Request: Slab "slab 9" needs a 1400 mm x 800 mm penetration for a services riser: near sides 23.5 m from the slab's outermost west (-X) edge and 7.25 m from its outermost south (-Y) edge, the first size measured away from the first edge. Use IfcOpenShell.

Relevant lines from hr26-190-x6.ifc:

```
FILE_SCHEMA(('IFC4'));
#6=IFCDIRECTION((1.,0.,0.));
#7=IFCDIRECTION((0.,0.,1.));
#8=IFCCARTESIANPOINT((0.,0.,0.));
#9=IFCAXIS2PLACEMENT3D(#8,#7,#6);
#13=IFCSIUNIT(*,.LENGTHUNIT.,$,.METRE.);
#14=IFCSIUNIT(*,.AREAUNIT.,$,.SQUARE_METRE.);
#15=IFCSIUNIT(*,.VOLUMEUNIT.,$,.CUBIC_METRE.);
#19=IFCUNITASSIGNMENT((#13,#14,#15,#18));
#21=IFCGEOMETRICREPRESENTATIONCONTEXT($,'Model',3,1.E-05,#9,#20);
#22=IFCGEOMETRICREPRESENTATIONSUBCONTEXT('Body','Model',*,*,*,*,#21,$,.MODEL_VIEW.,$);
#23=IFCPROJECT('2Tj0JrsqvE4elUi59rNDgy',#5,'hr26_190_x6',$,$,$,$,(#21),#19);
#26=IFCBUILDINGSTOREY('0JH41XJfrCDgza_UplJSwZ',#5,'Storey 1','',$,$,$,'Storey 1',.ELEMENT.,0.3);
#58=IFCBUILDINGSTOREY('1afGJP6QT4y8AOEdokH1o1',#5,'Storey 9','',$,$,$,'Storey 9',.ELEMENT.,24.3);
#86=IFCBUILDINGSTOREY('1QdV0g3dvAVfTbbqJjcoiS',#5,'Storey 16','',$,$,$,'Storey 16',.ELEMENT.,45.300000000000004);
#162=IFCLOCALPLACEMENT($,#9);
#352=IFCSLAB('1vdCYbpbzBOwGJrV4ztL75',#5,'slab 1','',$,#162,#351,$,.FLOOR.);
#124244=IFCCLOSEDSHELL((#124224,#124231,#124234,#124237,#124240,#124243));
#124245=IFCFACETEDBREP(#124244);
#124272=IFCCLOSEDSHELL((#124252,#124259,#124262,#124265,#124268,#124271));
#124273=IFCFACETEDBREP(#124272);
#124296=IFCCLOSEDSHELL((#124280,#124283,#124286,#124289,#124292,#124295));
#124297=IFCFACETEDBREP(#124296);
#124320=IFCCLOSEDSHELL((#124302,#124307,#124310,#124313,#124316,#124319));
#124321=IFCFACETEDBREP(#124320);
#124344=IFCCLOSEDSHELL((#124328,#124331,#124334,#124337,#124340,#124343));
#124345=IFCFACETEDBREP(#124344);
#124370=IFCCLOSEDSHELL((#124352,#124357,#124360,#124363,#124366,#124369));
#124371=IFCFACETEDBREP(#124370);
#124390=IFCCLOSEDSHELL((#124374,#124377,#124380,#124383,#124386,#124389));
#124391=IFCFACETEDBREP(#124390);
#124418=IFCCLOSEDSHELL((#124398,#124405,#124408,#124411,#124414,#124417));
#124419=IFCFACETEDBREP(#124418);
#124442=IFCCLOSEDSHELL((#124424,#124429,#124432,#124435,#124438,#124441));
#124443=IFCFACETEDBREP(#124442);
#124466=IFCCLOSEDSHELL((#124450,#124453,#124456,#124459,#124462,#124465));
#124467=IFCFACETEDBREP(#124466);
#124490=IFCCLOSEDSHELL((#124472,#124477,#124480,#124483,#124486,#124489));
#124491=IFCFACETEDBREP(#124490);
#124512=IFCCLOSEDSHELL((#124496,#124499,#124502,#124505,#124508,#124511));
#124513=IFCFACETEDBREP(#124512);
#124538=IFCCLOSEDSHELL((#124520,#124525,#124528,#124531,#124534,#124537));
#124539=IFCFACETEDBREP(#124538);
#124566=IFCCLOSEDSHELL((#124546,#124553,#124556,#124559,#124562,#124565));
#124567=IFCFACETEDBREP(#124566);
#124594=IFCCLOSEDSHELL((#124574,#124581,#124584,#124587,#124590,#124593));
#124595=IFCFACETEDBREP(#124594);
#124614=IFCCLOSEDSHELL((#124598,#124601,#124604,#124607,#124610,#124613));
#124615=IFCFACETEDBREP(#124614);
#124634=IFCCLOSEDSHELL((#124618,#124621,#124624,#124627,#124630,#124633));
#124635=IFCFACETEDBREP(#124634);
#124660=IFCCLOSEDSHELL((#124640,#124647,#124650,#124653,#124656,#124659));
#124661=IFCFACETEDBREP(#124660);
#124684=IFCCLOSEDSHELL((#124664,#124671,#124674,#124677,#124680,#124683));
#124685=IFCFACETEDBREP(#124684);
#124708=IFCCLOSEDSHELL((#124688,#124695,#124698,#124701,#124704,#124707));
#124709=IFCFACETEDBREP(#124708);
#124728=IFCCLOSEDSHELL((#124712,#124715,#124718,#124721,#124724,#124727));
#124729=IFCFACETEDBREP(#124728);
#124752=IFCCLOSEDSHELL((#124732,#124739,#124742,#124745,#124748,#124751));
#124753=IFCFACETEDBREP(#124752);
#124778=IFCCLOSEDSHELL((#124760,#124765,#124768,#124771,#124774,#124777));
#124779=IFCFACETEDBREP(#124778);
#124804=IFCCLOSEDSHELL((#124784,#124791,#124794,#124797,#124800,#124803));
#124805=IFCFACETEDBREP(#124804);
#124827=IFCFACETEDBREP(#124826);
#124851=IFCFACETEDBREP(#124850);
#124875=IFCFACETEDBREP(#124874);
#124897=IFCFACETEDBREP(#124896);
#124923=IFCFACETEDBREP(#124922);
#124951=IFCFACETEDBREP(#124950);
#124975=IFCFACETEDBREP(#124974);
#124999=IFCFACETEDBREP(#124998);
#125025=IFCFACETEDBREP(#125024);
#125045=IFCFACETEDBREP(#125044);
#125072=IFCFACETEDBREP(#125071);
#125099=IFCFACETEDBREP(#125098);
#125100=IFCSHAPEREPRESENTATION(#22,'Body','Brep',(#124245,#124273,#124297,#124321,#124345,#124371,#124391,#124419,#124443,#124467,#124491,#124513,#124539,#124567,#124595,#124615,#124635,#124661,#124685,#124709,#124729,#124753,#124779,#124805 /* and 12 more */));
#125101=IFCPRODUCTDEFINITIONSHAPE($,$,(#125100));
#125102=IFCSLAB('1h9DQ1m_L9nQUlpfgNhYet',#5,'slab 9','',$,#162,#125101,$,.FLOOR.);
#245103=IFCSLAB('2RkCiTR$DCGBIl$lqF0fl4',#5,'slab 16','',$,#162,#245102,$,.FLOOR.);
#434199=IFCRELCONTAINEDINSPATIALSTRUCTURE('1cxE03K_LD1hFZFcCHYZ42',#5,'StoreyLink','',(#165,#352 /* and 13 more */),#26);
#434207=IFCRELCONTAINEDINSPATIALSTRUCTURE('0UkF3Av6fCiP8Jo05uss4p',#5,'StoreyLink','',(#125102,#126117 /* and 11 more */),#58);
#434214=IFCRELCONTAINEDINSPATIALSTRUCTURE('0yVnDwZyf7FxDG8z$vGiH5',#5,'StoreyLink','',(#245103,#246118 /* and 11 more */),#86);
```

```python
import numpy as np
import ifcopenshell
import ifcopenshell.api.feature
import ifcopenshell.api.geometry
import ifcopenshell.api.root
import ifcopenshell.geom
import ifcopenshell.util.placement
import ifcopenshell.util.representation
import ifcopenshell.util.shape
import ifcopenshell.util.unit

model = ifcopenshell.open("hr26-190-x6.ifc")
unit_scale = ifcopenshell.util.unit.calculate_unit_scale(model)
settings = ifcopenshell.geom.settings()


def volume(element):
    """Net volume in cubic metres, openings subtracted."""
    shape = ifcopenshell.geom.create_shape(settings, element)
    return ifcopenshell.util.shape.get_volume(shape.geometry)


slab = model.by_guid("1h9DQ1m_L9nQUlpfgNhYet")
before = volume(slab)

# Extent in the slab's own axes, in metres. The edges named are its -X and -Y sides.
slab_shape = ifcopenshell.geom.create_shape(settings, slab)
vertices = ifcopenshell.util.shape.get_vertices(slab_shape.geometry)
x_min, y_min, bottom = vertices.min(axis=0)
top = vertices[:, 2].max()

opening = ifcopenshell.api.root.create_entity(model, ifc_class="IfcOpeningElement", name="Services riser opening", predefined_type="OPENING")
context = ifcopenshell.util.representation.get_context(model, "Model", "Body", "MODEL_VIEW")
width, depth = 1.4, 0.8
outline = [(0.0, 0.0), (width, 0.0), (width, depth), (0.0, depth), (0.0, 0.0)]
# Overshoot both faces by 50 mm so the cut is clean.
shape = ifcopenshell.api.geometry.add_slab_representation(
    model, context=context, depth=top - bottom + 0.1, polyline=outline
)
ifcopenshell.api.geometry.assign_representation(model, product=opening, representation=shape)

matrix = ifcopenshell.util.placement.get_local_placement(slab.ObjectPlacement)
matrix[:, 3] = matrix @ np.append(np.array([x_min + 23.5, y_min + 7.25, bottom - 0.05]) / unit_scale, 1.0)
ifcopenshell.api.geometry.edit_object_placement(model, product=opening, matrix=matrix, is_si=False)
ifcopenshell.api.feature.add_feature(model, feature=opening, element=slab)

after = volume(slab)

print(f"slab volume {before:.3f} -> {after:.3f} m3")

model.write("hr26-190-x6_rev.ifc")
```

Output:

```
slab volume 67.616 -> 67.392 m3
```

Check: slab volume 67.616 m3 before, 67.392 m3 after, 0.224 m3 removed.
